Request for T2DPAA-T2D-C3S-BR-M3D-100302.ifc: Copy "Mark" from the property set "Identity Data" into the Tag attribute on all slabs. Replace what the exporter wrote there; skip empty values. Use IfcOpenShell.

First a look at what the model holds.

```python
import ifcopenshell
import ifcopenshell.util.element

model = ifcopenshell.open("T2DPAA-T2D-C3S-BR-M3D-100302.ifc")
print(model.schema)
slabs = model.by_type("IfcSlab")
print(len(slabs), "slabs")
for e in slabs[:8]:
    source = ifcopenshell.util.element.get_pset(e, "Identity Data", "Mark")
    target = e.Tag
    print(e.id(), repr(source), repr(target), sep=" | ")
```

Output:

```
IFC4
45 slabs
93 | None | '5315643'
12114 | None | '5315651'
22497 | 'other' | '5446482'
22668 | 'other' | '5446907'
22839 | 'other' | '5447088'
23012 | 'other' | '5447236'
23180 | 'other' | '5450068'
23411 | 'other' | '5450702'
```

```python
import ifcopenshell
import ifcopenshell.util.element

model = ifcopenshell.open("T2DPAA-T2D-C3S-BR-M3D-100302.ifc")

count = 0
for e in model.by_type("IfcSlab"):
    value = ifcopenshell.util.element.get_pset(e, "Identity Data", "Mark")
    current = e.Tag
    if not value or not value.strip() or current == value:
        continue
    e.Tag = value
    count += 1

print(count, "slabs updated")

model.write("T2DPAA-T2D-C3S-BR-M3D-100302-out.ifc")
```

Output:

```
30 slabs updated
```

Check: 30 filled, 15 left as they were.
